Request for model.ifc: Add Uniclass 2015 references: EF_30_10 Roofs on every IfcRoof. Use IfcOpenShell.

First a look at what the model holds.

```python
import ifcopenshell

model = ifcopenshell.open("model.ifc")
print(model.schema)
print("classifications:", [c.Name for c in model.by_type("IfcClassification")])
for ifc_class in ("IfcDoor", "IfcRoof", "IfcStair", "IfcWall", "IfcWindow"):
    print(ifc_class, len(model.by_type(ifc_class)))
```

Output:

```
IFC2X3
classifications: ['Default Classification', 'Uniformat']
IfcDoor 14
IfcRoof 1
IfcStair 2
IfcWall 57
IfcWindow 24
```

```python
import ifcopenshell
import ifcopenshell.api.classification

model = ifcopenshell.open("model.ifc")

# IFC2X3 requires Source and Edition and has no link from the project to the system.
system = model.create_entity("IfcClassification", Source="NBS", Edition="2015", Name="Uniclass 2015")

codes = {
    "IfcRoof": ("EF_30_10", "Roofs"),
}
for ifc_class, (code, name) in codes.items():
    products = model.by_type(ifc_class)
    ifcopenshell.api.classification.add_reference(
        model, products=products, classification=system, identification=code, name=name
    )
    print(code, len(products))

model.write("model_edited.ifc")
```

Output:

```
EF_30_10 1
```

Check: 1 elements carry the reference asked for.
